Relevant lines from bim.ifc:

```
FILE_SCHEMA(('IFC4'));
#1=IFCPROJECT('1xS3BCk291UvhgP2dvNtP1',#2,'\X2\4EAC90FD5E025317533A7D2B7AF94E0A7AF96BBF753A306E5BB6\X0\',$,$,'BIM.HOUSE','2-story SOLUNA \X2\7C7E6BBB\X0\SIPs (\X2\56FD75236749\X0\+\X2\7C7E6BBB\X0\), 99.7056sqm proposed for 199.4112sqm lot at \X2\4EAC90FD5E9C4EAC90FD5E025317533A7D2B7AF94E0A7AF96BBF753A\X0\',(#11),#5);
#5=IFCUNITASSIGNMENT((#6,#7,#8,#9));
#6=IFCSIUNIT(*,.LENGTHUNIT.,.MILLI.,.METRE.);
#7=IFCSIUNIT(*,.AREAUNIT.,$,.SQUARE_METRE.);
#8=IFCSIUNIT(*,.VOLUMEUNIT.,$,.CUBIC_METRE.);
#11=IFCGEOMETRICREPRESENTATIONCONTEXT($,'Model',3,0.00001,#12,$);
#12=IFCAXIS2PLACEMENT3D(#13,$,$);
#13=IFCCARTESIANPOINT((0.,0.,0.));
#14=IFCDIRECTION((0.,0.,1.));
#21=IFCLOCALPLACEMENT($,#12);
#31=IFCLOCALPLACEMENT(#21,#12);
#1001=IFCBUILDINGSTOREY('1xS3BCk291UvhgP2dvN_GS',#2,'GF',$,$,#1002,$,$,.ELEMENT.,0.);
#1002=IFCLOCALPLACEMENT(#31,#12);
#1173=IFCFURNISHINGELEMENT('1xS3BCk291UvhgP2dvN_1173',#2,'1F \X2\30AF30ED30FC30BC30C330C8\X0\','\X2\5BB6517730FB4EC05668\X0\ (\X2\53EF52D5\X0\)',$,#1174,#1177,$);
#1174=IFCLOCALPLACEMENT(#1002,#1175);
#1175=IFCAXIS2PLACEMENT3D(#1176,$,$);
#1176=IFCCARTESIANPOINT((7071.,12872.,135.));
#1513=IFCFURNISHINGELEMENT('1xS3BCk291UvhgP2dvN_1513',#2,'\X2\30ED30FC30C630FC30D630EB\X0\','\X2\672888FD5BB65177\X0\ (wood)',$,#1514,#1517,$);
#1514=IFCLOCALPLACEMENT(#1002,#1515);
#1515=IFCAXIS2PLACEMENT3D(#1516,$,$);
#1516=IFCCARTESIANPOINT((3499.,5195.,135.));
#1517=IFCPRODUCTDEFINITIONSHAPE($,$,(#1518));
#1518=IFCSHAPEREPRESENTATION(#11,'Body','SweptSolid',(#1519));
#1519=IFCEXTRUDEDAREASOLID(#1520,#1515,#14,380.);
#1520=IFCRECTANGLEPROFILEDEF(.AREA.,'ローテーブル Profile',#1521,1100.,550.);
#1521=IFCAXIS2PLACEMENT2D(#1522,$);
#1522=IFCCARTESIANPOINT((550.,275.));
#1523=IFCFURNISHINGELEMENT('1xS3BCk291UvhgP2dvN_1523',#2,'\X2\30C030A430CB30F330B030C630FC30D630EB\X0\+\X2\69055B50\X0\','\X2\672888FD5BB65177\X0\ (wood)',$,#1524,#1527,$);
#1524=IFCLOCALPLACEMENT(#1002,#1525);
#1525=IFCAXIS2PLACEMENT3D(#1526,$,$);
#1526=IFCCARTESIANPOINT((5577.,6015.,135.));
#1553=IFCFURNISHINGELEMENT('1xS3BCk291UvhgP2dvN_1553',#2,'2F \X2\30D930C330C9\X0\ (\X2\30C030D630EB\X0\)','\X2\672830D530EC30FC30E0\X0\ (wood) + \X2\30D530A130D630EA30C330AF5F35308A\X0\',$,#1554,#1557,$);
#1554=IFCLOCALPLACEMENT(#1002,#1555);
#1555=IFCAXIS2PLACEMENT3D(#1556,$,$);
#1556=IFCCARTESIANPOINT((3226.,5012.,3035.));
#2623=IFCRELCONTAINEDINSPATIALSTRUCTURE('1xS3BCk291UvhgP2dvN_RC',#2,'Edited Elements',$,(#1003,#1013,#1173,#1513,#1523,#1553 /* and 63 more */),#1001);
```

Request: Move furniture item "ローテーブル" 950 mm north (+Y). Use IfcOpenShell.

```python
import ifcopenshell
import ifcopenshell.api.geometry
import ifcopenshell.util.placement

model = ifcopenshell.open("bim.ifc")

item = model.by_guid("1xS3BCk291UvhgP2dvN_1513")
matrix = ifcopenshell.util.placement.get_local_placement(item.ObjectPlacement)
matrix[1, 3] += 950.0
ifcopenshell.api.geometry.edit_object_placement(model, product=item, matrix=matrix, is_si=False)

print(ifcopenshell.util.placement.get_local_placement(item.ObjectPlacement).round(3) + 0.0)

model.write("bim-out.ifc")
```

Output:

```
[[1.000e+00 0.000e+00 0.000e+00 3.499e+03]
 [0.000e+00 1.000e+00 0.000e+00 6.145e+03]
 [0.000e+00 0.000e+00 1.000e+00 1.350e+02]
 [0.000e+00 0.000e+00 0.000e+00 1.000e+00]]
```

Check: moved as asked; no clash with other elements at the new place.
